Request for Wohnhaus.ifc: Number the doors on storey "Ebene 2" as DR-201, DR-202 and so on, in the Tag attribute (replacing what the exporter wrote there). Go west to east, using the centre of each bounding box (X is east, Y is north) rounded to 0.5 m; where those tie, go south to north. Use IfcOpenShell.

First a look at what the model holds.

```python
import ifcopenshell
import ifcopenshell.util.element
import ifcopenshell.util.placement

model = ifcopenshell.open("Wohnhaus.ifc")
print(model.schema)
storey = next(s for s in model.by_type("IfcBuildingStorey") if s.Name == "Ebene 2")
doors = [e for e in ifcopenshell.util.element.get_decomposition(storey) if e.is_a("IfcDoor")]
for e in sorted(doors, key=lambda e: e.id()):
    origin = ifcopenshell.util.placement.get_local_placement(e.ObjectPlacement)[:3, 3]
    print(e.id(), e.Tag, e.Name, origin.round(2) + 0.0, sep=" | ")
```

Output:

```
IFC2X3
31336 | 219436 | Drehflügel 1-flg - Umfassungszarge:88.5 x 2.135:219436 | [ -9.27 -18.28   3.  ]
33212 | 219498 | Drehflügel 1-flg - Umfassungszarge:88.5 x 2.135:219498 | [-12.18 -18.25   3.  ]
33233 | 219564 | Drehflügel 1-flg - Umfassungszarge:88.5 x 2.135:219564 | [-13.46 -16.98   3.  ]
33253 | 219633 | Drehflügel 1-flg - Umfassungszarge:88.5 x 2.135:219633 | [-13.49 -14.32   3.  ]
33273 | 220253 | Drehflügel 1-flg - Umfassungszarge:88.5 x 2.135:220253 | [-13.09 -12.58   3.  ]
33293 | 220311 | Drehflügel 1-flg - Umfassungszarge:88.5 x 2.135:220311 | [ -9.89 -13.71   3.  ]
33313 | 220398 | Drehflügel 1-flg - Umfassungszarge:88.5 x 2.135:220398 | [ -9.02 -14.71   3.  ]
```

```python
import ifcopenshell
import ifcopenshell.geom
import ifcopenshell.util.element
import ifcopenshell.util.shape

model = ifcopenshell.open("Wohnhaus.ifc")
settings = ifcopenshell.geom.settings()
settings.set("use-world-coords", True)


def centre(element):
    shape = ifcopenshell.geom.create_shape(settings, element)
    return ifcopenshell.util.shape.get_bbox_centroid(shape.geometry)


storey = next(s for s in model.by_type("IfcBuildingStorey") if s.Name == "Ebene 2")
doors = [e for e in ifcopenshell.util.element.get_decomposition(storey) if e.is_a("IfcDoor")]

# Insertion points can sit at a corner or the storey origin, so sort by the geometry (in metres).
centres = {e: centre(e) for e in doors}
doors.sort(key=lambda e: (round(centres[e][0] / 0.5), centres[e][1]))

for i, e in enumerate(doors, start=1):
    number = f"DR-2{i:02d}"
    e.Tag = number
    print(e.id(), number)

model.write("Wohnhaus_edited.ifc")
```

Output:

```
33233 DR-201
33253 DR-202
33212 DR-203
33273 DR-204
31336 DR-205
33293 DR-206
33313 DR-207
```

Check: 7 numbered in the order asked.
